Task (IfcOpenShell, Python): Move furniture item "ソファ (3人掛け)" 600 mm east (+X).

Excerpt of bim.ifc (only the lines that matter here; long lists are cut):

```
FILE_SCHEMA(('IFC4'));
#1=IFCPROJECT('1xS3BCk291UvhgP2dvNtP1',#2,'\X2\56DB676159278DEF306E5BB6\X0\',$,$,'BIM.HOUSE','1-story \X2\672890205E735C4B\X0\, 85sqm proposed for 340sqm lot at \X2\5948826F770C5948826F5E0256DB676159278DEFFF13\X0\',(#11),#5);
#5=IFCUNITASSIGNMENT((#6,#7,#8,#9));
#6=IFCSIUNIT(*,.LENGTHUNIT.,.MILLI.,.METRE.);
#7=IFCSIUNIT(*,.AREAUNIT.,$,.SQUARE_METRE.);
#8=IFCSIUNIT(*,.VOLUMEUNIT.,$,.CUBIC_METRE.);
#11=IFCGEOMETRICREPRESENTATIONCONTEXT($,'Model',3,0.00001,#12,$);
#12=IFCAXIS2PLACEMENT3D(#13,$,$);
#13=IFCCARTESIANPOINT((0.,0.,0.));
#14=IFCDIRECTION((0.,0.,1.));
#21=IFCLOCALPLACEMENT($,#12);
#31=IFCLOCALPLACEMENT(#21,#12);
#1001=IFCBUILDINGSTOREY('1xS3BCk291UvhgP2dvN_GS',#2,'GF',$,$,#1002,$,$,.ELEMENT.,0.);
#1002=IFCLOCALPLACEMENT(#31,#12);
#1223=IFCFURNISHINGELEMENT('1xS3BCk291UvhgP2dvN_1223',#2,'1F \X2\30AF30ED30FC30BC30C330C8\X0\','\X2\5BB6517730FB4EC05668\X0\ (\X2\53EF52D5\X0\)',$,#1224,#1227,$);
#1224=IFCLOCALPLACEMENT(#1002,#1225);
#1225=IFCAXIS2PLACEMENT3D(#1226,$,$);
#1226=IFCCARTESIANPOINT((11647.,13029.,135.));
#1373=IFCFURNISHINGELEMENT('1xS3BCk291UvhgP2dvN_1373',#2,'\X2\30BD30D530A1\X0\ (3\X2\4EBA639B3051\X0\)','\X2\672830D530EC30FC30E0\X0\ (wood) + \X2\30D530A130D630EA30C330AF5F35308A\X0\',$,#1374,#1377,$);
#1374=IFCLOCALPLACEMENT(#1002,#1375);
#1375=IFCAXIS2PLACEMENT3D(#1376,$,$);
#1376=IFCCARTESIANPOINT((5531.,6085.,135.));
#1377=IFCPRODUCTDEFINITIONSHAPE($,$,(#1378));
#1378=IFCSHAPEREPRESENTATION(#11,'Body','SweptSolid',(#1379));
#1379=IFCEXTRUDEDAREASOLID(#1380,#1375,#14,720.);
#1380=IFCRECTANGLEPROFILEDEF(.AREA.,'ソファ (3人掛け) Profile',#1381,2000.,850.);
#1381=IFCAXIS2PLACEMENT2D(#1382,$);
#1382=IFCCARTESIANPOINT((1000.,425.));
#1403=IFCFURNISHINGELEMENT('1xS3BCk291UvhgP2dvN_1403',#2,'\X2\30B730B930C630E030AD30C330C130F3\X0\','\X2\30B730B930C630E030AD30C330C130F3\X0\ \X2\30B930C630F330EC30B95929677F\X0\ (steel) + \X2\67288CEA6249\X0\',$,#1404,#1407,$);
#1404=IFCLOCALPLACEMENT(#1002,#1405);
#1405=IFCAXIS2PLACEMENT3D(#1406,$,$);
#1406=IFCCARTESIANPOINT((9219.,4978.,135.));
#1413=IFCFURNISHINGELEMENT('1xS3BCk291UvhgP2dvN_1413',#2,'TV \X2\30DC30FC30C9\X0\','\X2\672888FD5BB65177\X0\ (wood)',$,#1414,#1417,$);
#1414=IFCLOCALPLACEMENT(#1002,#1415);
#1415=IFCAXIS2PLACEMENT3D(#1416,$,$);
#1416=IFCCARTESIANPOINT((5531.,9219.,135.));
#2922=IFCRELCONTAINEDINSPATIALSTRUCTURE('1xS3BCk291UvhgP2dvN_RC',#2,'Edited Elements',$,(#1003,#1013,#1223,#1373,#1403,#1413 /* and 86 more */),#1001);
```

```python
import ifcopenshell
import ifcopenshell.api.geometry
import ifcopenshell.util.placement

model = ifcopenshell.open("bim.ifc")

item = model.by_guid("1xS3BCk291UvhgP2dvN_1373")
matrix = ifcopenshell.util.placement.get_local_placement(item.ObjectPlacement)
matrix[0, 3] += 600.0
ifcopenshell.api.geometry.edit_object_placement(model, product=item, matrix=matrix, is_si=False)

print(ifcopenshell.util.placement.get_local_placement(item.ObjectPlacement).round(3) + 0.0)

model.write("bim_rev.ifc")
```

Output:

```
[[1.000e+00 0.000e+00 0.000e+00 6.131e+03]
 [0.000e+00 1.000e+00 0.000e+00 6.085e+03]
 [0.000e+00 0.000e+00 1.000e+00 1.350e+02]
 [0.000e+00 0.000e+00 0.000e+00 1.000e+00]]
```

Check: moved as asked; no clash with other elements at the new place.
